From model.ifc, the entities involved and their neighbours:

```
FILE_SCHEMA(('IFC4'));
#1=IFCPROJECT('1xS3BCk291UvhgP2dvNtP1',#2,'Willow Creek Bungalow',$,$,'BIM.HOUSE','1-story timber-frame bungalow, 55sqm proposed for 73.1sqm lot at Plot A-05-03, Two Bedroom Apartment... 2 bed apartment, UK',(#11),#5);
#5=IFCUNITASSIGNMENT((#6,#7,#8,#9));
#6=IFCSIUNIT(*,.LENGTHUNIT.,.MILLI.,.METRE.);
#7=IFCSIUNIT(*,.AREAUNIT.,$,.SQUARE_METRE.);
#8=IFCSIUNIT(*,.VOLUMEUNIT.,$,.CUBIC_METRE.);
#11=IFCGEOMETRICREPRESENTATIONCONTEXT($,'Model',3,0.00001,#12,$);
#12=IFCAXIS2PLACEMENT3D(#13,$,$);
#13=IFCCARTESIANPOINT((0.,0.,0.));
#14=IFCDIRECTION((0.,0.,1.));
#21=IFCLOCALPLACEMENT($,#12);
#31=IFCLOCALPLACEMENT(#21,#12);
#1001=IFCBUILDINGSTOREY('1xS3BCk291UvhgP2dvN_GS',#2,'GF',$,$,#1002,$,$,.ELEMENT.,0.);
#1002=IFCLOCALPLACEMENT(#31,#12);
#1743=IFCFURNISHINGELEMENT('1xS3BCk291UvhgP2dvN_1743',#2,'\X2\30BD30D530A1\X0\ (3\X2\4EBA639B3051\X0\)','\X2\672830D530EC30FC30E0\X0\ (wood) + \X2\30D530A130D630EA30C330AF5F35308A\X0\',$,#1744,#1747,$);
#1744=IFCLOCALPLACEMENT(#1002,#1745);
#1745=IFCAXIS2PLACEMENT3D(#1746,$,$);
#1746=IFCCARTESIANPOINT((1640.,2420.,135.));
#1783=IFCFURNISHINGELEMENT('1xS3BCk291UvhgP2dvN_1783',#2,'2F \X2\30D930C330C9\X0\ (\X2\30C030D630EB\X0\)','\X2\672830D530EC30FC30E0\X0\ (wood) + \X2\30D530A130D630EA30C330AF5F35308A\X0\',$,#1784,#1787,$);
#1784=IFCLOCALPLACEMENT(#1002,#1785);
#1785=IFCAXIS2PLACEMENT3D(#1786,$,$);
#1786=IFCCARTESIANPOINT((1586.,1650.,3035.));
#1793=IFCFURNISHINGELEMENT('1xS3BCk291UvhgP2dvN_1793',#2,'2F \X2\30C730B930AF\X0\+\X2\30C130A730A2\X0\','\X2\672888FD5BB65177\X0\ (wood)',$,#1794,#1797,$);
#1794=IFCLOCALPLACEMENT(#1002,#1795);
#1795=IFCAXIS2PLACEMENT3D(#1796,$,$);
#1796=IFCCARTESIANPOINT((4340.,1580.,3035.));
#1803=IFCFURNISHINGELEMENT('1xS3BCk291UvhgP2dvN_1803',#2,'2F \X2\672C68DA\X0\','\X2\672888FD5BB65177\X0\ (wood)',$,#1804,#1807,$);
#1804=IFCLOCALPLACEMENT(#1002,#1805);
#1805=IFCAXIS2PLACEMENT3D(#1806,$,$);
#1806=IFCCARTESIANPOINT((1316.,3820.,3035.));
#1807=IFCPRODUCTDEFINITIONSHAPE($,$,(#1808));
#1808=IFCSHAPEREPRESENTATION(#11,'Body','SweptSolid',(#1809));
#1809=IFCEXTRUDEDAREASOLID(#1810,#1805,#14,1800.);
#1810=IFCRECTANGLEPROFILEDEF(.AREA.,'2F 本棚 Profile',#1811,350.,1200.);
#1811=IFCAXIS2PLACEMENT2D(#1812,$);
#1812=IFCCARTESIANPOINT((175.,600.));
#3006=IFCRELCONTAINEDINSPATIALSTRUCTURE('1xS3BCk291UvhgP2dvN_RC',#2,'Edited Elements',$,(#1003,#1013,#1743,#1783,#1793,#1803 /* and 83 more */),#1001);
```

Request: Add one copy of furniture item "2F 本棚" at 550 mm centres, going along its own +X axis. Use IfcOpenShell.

```python
import ifcopenshell
import ifcopenshell.api.geometry
import ifcopenshell.api.root
import ifcopenshell.util.element
import ifcopenshell.util.placement
import ifcopenshell.util.unit

model = ifcopenshell.open("model.ifc")
unit_scale = ifcopenshell.util.unit.calculate_unit_scale(model)


def reuse_history(source, copy):
    """copy_class also copies each property set's owner history, people and application; keep the originals."""
    for rel in copy.IsDefinedBy:
        if rel.is_a("IfcRelDefinesByProperties") and (history := rel.RelatingPropertyDefinition.OwnerHistory):
            rel.RelatingPropertyDefinition.OwnerHistory = source.OwnerHistory
            ifcopenshell.util.element.remove_deep2(model, history)


source = model.by_guid("1xS3BCk291UvhgP2dvN_1803")
base = ifcopenshell.util.placement.get_local_placement(source.ObjectPlacement)
step = base[:3, 0] * 0.55 / unit_scale

for i in range(1, 2):
    copy = ifcopenshell.api.root.copy_class(model, product=source)
    copy.Representation = ifcopenshell.util.element.copy_deep(
        model, source.Representation, exclude=["IfcGeometricRepresentationContext", "IfcRepresentationMap"]
    )
    reuse_history(source, copy)
    matrix = base.copy()
    matrix[:3, 3] += i * step
    print("added at", matrix[:3, 3].round(3) + 0.0)
    ifcopenshell.api.geometry.edit_object_placement(model, product=copy, matrix=matrix, is_si=False)

model.write("model_v2.ifc")
```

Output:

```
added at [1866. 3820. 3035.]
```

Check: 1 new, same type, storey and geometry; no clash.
